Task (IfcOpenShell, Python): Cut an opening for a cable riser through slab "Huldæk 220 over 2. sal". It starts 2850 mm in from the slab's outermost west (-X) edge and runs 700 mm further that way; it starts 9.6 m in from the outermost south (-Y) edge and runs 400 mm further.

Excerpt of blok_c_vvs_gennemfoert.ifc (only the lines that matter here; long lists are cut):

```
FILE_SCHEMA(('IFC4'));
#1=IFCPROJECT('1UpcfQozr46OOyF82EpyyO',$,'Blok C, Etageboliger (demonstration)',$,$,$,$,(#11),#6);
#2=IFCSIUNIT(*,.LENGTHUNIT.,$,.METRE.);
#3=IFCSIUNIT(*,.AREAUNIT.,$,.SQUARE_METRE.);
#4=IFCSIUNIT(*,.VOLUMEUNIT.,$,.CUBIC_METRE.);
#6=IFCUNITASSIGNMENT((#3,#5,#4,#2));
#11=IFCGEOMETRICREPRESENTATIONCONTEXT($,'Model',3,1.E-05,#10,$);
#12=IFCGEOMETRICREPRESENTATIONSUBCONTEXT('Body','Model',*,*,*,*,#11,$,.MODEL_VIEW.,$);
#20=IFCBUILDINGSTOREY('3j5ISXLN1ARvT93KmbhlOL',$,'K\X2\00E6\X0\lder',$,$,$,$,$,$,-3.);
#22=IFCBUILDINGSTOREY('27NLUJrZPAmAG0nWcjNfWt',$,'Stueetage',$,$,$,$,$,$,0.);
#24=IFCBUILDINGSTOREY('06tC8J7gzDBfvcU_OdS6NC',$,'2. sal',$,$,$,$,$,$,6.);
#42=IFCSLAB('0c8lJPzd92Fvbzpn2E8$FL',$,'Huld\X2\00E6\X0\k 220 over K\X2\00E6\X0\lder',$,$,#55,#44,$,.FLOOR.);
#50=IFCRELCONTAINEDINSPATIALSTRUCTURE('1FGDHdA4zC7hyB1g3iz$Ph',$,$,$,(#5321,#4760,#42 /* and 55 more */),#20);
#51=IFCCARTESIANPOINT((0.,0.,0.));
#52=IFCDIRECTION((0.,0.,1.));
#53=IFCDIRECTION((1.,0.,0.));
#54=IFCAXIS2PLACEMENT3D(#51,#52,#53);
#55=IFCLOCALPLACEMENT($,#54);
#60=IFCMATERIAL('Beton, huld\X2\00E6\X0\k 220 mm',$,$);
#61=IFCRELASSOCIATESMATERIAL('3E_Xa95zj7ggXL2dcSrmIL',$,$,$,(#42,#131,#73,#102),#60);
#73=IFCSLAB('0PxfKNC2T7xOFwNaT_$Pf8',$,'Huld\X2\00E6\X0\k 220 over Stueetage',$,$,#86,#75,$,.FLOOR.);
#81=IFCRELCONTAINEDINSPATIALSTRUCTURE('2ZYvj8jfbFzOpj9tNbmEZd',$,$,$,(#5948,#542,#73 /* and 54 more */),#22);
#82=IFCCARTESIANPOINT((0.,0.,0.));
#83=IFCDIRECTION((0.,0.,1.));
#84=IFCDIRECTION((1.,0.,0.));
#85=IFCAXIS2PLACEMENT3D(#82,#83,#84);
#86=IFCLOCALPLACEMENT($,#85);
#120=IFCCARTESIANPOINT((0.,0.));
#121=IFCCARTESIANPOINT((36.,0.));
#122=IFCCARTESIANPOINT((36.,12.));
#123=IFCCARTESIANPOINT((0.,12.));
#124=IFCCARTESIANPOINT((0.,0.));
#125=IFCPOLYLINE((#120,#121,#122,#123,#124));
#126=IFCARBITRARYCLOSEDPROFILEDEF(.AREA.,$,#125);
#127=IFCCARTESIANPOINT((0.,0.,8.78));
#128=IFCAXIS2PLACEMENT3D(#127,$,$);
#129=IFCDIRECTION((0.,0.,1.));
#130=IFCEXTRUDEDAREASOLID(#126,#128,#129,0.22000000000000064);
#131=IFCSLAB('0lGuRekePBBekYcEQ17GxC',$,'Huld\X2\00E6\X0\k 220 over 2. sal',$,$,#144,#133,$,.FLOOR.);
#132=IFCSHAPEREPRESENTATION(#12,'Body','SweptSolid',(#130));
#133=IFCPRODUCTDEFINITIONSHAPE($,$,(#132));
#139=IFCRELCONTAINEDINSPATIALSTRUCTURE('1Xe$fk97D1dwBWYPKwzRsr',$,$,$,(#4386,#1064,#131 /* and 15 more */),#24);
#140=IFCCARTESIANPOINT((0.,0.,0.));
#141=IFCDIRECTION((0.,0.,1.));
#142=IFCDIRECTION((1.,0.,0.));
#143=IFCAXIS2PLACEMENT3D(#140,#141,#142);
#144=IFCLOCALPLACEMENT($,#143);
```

```python
import numpy as np
import ifcopenshell
import ifcopenshell.api.feature
import ifcopenshell.api.geometry
import ifcopenshell.api.root
import ifcopenshell.geom
import ifcopenshell.util.placement
import ifcopenshell.util.representation
import ifcopenshell.util.shape
import ifcopenshell.util.unit

model = ifcopenshell.open("blok_c_vvs_gennemfoert.ifc")
unit_scale = ifcopenshell.util.unit.calculate_unit_scale(model)
settings = ifcopenshell.geom.settings()


def volume(element):
    """Net volume in cubic metres, openings subtracted."""
    shape = ifcopenshell.geom.create_shape(settings, element)
    return ifcopenshell.util.shape.get_volume(shape.geometry)


slab = model.by_id(131)
before = volume(slab)

# Extent in the slab's own axes, in metres. The edges named are its -X and -Y sides.
slab_shape = ifcopenshell.geom.create_shape(settings, slab)
vertices = ifcopenshell.util.shape.get_vertices(slab_shape.geometry)
x_min, y_min, bottom = vertices.min(axis=0)
top = vertices[:, 2].max()

opening = ifcopenshell.api.root.create_entity(model, ifc_class="IfcOpeningElement", name="Cable riser opening", predefined_type="OPENING")
context = ifcopenshell.util.representation.get_context(model, "Model", "Body", "MODEL_VIEW")
width, depth = 0.7, 0.4
outline = [(0.0, 0.0), (width, 0.0), (width, depth), (0.0, depth), (0.0, 0.0)]
# Overshoot both faces by 50 mm so the cut is clean.
shape = ifcopenshell.api.geometry.add_slab_representation(
    model, context=context, depth=top - bottom + 0.1, polyline=outline
)
ifcopenshell.api.geometry.assign_representation(model, product=opening, representation=shape)

matrix = ifcopenshell.util.placement.get_local_placement(slab.ObjectPlacement)
matrix[:, 3] = matrix @ np.append(np.array([x_min + 2.85, y_min + 9.6, bottom - 0.05]) / unit_scale, 1.0)
ifcopenshell.api.geometry.edit_object_placement(model, product=opening, matrix=matrix, is_si=False)
ifcopenshell.api.feature.add_feature(model, feature=opening, element=slab)

after = volume(slab)

print(f"slab volume {before:.3f} -> {after:.3f} m3")

model.write("blok_c_vvs_gennemfoert_v2.ifc")
```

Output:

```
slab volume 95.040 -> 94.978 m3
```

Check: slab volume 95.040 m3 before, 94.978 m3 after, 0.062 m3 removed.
